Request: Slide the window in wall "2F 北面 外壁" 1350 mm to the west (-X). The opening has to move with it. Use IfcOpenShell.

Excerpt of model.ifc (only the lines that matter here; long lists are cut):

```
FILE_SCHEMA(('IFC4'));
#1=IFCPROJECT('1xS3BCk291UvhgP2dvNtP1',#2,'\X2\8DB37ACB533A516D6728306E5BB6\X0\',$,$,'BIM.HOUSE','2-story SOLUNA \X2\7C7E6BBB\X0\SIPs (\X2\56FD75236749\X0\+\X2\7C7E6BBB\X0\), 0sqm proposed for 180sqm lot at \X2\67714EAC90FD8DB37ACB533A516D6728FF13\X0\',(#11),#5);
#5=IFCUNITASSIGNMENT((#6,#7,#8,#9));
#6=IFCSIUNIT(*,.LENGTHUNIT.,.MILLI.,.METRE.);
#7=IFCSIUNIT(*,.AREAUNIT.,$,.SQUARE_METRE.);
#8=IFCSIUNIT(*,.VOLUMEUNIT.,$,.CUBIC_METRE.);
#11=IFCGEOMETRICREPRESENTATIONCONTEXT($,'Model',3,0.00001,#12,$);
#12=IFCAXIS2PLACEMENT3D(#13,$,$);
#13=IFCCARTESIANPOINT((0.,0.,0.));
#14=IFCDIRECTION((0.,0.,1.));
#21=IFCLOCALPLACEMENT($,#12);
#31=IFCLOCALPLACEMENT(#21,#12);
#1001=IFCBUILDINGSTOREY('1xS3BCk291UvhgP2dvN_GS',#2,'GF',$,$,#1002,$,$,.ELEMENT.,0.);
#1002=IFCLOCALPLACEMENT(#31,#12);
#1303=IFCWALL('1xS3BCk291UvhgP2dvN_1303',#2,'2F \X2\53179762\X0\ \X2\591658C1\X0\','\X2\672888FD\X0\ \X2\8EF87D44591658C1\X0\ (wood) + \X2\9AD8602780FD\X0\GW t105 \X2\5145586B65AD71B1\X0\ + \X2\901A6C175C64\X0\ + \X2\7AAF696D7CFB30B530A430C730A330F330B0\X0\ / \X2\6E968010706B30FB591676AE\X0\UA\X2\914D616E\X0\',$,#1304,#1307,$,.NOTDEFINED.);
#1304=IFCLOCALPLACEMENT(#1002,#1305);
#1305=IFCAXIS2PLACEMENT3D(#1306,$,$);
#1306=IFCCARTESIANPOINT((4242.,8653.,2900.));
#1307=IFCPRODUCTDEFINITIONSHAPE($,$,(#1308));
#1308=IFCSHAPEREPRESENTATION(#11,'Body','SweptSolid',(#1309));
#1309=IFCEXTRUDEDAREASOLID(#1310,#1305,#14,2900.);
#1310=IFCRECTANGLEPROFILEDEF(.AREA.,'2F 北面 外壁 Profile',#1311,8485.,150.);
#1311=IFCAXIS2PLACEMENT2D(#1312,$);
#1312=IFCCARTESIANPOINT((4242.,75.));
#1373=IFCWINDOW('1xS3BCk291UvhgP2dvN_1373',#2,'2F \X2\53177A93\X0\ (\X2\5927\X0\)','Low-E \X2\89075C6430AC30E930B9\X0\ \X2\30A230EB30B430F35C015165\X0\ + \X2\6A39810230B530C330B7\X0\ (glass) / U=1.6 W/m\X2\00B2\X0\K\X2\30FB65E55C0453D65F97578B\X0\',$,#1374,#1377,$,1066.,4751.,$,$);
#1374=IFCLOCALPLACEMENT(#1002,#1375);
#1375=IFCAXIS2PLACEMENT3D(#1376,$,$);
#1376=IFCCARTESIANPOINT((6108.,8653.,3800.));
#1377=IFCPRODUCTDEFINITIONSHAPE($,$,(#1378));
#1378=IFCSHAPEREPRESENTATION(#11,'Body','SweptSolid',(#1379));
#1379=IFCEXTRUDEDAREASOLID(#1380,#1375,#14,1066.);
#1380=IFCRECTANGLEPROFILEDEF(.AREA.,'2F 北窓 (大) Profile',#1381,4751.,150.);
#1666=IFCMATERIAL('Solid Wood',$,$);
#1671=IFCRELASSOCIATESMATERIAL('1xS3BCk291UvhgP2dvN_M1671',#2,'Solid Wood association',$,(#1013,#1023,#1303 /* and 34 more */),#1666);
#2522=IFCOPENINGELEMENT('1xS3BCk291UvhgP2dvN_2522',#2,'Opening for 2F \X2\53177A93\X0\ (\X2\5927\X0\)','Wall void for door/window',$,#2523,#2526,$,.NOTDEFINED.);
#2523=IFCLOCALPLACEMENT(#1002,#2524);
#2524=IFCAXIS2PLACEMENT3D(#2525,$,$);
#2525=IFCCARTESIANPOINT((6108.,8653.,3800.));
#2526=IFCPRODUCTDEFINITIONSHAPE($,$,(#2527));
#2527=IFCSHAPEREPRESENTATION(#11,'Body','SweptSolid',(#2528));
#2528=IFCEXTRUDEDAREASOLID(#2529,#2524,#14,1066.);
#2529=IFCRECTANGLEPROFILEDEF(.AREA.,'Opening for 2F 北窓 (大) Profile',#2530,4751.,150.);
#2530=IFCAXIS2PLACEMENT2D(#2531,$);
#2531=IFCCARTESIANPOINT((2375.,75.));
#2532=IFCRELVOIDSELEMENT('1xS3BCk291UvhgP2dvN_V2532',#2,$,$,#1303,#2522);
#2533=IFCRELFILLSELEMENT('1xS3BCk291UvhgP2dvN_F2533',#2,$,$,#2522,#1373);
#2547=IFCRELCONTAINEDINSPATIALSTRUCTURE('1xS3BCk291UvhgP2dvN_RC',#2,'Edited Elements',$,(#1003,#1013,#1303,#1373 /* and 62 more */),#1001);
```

```python
import ifcopenshell
import ifcopenshell.api.geometry
import ifcopenshell.util.placement
import ifcopenshell.util.unit

model = ifcopenshell.open("model.ifc")
unit_scale = ifcopenshell.util.unit.calculate_unit_scale(model)

window = model.by_guid("1xS3BCk291UvhgP2dvN_1373")
opening = window.FillsVoids[0].RelatingOpeningElement
wall = opening.VoidsElements[0].RelatingBuildingElement

wall_matrix = ifcopenshell.util.placement.get_local_placement(wall.ObjectPlacement)
shift = wall_matrix[:3, 0] * -1.35 / unit_scale
before = ifcopenshell.util.placement.get_local_placement(window.ObjectPlacement)[:3, 3].copy()

# The window is not placed relative to its opening, so move both.
for product in (opening, window):
    matrix = ifcopenshell.util.placement.get_local_placement(product.ObjectPlacement)
    matrix[:3, 3] += shift
    ifcopenshell.api.geometry.edit_object_placement(model, product=product, matrix=matrix, is_si=False)

after = ifcopenshell.util.placement.get_local_placement(window.ObjectPlacement)[:3, 3]
print("window moved by", (after - before).round(3) + 0.0)

model.write("model_v2.ifc")
```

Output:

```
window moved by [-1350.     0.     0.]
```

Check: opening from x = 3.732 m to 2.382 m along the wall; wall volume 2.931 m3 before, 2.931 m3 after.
